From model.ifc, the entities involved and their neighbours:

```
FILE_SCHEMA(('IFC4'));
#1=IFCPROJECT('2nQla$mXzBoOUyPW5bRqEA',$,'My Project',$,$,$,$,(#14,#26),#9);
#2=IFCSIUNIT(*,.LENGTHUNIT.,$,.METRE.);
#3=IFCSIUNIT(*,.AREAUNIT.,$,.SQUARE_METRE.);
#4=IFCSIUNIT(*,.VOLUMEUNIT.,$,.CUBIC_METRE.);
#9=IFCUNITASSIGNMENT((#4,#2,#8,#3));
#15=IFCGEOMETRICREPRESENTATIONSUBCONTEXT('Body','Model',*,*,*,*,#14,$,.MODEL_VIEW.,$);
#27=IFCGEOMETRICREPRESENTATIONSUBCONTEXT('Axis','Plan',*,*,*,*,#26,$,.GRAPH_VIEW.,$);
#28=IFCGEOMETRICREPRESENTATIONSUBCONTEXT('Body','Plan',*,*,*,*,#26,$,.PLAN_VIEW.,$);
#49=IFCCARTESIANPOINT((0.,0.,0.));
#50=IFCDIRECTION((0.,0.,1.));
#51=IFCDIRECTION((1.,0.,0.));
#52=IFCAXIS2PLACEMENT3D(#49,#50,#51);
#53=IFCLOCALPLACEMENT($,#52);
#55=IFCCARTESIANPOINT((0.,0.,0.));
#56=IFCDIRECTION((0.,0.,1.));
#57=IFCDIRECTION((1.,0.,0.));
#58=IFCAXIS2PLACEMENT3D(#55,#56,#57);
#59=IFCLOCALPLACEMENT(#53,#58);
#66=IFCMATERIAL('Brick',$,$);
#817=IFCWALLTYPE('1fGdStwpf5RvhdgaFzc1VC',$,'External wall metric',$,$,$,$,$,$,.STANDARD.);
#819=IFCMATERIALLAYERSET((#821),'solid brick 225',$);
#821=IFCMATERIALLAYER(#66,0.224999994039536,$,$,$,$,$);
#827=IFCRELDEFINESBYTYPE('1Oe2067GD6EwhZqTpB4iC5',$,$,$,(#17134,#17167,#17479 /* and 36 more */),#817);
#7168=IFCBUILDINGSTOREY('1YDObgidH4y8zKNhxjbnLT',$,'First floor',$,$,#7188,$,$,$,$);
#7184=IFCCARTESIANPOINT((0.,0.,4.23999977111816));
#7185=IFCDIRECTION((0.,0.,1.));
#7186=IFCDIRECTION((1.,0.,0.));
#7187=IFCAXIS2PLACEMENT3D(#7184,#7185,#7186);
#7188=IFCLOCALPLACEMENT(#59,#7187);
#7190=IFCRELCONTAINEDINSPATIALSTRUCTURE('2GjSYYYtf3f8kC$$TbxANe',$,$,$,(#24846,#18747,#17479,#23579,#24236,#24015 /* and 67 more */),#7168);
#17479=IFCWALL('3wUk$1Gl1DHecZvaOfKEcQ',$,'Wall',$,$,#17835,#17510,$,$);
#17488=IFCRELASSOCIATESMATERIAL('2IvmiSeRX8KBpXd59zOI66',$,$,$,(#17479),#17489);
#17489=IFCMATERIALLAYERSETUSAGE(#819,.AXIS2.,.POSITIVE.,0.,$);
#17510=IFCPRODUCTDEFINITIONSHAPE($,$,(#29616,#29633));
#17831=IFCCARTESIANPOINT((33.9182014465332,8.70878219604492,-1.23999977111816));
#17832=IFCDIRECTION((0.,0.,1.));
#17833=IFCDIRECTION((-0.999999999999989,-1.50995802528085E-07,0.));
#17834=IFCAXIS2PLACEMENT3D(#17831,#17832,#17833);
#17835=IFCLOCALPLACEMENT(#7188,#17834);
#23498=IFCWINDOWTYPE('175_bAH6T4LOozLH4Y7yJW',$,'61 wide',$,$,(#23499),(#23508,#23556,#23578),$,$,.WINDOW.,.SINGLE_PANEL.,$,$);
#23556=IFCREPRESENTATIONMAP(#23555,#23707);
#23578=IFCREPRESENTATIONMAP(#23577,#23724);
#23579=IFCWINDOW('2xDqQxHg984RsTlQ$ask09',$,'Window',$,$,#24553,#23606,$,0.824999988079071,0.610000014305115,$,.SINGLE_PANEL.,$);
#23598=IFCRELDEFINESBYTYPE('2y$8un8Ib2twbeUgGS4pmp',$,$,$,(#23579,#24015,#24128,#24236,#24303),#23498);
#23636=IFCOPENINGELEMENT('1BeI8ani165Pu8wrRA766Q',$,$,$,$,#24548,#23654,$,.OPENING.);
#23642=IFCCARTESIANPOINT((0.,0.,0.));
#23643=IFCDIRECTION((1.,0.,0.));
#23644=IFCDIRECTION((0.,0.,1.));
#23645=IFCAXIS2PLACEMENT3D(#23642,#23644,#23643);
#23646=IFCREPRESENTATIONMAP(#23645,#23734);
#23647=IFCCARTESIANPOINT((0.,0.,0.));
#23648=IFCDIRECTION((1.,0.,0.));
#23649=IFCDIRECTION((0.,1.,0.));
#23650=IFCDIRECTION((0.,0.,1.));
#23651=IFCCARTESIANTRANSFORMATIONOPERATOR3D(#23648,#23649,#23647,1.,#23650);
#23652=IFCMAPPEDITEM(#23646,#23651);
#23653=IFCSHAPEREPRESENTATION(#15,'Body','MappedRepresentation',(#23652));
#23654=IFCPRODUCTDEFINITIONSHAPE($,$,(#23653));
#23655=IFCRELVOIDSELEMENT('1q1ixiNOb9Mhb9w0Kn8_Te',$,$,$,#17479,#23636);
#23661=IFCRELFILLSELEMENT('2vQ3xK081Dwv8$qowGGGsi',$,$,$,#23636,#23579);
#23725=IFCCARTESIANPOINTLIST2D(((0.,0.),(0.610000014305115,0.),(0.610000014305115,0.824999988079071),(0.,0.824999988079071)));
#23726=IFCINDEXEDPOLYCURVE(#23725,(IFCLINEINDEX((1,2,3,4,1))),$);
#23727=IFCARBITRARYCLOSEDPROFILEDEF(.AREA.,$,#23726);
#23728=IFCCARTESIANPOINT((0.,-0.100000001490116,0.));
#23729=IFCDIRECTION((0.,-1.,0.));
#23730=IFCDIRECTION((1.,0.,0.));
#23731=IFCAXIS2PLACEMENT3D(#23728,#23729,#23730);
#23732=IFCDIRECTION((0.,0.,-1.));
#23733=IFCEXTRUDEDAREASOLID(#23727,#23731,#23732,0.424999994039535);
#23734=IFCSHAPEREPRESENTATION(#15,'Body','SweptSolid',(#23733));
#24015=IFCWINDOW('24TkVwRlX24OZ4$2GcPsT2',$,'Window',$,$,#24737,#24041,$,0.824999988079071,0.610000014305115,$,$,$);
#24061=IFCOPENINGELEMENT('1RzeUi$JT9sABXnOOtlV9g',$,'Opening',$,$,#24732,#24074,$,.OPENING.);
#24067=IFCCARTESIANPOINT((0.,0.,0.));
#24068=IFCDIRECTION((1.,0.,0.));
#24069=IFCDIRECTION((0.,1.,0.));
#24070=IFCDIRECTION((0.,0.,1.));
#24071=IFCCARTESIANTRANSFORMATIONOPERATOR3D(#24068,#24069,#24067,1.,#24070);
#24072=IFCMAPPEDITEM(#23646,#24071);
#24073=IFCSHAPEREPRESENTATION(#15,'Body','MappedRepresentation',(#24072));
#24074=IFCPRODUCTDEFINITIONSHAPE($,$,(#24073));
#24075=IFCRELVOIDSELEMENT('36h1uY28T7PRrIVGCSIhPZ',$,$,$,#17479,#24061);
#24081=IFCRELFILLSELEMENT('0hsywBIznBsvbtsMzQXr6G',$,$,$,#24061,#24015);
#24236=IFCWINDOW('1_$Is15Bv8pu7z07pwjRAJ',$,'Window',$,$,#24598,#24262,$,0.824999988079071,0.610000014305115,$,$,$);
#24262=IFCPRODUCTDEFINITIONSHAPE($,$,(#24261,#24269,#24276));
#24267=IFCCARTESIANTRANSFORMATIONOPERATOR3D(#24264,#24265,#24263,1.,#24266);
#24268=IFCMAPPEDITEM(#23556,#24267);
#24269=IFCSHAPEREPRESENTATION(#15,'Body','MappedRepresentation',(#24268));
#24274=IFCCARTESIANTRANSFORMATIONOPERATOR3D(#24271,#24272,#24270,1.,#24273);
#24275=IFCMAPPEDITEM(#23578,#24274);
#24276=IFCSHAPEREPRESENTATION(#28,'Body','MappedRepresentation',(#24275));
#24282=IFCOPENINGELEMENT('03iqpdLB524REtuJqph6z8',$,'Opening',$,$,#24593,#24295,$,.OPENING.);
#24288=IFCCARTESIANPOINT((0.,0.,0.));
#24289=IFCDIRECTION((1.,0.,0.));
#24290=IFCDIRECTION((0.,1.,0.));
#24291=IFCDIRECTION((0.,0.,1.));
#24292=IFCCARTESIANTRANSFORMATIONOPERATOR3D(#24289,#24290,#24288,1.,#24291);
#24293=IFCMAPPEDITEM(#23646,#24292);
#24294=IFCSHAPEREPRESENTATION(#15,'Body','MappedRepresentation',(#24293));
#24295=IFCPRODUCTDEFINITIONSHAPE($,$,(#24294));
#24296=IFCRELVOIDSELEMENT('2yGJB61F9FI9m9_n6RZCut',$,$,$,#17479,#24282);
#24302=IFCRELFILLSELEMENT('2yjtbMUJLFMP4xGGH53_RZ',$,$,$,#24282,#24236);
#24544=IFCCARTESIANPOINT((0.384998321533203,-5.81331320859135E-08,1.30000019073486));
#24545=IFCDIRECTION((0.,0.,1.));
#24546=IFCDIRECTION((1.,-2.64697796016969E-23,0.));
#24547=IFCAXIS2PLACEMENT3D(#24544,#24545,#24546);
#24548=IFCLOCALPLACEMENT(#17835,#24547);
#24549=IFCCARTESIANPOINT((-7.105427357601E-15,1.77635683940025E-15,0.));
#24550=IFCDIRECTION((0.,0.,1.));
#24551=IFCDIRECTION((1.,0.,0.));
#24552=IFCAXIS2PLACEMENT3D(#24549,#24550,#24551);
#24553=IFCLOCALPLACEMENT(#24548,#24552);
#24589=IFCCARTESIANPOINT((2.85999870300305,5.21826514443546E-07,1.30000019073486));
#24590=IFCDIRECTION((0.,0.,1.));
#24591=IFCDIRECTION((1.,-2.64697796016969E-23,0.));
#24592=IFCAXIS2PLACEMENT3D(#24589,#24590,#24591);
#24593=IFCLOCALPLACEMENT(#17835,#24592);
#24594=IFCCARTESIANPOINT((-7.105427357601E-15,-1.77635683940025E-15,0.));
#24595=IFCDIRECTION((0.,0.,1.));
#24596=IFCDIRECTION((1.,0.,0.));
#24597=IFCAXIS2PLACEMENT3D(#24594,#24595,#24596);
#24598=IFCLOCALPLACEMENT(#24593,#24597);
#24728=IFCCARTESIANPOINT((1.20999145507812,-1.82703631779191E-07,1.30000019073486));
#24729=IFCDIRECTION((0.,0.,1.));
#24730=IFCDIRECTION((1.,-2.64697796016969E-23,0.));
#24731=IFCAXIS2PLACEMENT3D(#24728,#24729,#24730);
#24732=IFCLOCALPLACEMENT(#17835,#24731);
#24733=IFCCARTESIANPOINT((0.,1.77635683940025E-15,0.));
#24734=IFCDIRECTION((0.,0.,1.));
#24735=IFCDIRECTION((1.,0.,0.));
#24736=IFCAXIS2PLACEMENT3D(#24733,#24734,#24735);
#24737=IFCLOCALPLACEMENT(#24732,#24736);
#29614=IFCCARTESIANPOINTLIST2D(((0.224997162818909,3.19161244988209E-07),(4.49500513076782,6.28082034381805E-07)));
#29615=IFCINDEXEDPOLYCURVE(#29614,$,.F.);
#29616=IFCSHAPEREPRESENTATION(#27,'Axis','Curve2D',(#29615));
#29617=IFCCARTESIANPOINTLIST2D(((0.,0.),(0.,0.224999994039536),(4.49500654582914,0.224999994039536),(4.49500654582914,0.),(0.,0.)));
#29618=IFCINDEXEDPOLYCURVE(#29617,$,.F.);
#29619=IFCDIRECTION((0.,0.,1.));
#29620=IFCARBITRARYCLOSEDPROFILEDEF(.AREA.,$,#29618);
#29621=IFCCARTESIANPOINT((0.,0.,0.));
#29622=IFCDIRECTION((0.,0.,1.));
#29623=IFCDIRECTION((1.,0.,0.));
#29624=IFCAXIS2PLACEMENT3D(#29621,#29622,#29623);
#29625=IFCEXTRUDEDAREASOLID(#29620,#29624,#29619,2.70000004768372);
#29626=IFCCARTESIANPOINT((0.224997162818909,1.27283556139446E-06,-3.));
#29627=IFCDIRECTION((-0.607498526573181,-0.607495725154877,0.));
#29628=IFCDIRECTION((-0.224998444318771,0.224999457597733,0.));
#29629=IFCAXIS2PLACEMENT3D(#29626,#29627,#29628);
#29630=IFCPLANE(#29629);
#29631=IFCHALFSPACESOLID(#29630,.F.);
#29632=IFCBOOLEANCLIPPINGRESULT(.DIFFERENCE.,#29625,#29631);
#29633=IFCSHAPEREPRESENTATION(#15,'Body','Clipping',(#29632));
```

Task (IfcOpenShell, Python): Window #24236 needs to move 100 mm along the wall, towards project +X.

```python
import ifcopenshell
import ifcopenshell.api.geometry
import ifcopenshell.util.placement
import ifcopenshell.util.unit

model = ifcopenshell.open("model.ifc")
unit_scale = ifcopenshell.util.unit.calculate_unit_scale(model)

window = model.by_id(24236)
opening = window.FillsVoids[0].RelatingOpeningElement
wall = opening.VoidsElements[0].RelatingBuildingElement

wall_matrix = ifcopenshell.util.placement.get_local_placement(wall.ObjectPlacement)
shift = wall_matrix[:3, 0] * -0.1 / unit_scale
before = ifcopenshell.util.placement.get_local_placement(window.ObjectPlacement)[:3, 3].copy()

# The window is placed relative to its opening, so it follows when the opening moves.
matrix = ifcopenshell.util.placement.get_local_placement(opening.ObjectPlacement)
matrix[:3, 3] += shift
ifcopenshell.api.geometry.edit_object_placement(
    model, product=opening, matrix=matrix, is_si=False, should_transform_children=True
)

after = ifcopenshell.util.placement.get_local_placement(window.ObjectPlacement)[:3, 3]
print("window moved by", (after - before).round(3) + 0.0)

model.write("model-out.ifc")
```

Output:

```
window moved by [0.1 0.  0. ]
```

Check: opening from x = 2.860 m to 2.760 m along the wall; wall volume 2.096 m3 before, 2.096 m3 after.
